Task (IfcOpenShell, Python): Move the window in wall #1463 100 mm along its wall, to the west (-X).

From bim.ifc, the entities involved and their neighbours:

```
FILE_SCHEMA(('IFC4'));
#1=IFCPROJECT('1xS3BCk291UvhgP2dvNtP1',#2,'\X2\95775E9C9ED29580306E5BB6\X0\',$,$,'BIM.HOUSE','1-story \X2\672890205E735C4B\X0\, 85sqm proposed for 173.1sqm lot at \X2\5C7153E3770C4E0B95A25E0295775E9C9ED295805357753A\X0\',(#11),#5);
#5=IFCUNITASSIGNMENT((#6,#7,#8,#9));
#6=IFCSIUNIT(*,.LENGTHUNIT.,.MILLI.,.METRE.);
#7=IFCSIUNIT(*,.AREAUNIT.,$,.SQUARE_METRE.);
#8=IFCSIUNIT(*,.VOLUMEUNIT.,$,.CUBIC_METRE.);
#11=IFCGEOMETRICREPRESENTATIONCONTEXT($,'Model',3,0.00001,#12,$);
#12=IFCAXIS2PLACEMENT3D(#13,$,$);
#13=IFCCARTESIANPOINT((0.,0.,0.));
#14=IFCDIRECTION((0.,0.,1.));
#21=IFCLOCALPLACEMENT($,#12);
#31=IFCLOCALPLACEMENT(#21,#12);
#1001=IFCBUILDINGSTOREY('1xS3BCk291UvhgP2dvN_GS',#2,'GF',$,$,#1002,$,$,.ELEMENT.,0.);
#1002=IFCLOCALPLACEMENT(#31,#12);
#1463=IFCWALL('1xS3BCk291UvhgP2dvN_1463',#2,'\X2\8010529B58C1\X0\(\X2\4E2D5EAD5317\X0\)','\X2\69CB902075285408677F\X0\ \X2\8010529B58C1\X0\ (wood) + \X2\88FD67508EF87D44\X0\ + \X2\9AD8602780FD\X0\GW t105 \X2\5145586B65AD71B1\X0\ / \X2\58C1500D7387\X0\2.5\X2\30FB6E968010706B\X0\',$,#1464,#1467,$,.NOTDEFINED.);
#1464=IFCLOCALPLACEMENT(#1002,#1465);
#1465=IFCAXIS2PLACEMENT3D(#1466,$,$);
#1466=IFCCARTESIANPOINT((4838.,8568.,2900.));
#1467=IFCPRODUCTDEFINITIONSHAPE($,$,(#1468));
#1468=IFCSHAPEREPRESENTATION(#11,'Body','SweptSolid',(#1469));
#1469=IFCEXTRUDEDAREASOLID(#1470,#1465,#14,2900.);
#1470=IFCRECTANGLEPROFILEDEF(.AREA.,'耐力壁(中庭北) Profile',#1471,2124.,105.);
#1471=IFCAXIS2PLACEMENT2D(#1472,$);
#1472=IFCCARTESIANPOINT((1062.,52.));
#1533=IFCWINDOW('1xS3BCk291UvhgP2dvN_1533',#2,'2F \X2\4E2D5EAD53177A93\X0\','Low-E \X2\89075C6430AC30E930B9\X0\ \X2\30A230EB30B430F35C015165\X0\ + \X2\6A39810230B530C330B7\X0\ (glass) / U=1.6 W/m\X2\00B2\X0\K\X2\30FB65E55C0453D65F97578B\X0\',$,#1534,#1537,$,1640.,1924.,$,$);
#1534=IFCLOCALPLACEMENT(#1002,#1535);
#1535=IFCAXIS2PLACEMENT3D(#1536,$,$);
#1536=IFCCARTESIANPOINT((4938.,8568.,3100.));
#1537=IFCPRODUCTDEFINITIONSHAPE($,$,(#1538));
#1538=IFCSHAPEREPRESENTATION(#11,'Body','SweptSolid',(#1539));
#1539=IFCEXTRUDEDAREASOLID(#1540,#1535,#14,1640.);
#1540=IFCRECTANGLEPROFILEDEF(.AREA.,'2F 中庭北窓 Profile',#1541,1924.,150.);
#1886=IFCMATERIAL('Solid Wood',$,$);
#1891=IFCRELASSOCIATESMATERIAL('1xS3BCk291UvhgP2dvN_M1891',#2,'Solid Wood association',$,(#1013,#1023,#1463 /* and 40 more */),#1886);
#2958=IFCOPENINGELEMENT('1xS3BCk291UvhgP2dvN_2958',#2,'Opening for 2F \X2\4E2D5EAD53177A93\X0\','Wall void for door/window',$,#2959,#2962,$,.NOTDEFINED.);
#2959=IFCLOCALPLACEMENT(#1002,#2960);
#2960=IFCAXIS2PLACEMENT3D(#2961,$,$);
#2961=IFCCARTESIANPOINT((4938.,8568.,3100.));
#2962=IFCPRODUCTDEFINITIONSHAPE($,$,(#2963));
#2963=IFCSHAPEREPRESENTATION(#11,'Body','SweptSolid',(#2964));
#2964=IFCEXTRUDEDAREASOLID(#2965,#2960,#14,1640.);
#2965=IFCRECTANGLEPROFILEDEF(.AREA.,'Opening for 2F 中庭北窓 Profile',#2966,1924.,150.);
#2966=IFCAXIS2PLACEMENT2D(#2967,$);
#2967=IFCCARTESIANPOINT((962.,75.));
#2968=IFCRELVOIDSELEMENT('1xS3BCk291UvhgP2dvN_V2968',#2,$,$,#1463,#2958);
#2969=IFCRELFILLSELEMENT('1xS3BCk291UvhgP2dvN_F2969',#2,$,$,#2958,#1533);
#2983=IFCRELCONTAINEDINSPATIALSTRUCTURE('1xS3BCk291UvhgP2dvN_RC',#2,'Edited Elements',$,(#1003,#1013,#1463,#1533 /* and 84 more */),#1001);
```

```python
import ifcopenshell
import ifcopenshell.api.geometry
import ifcopenshell.util.placement
import ifcopenshell.util.unit

model = ifcopenshell.open("bim.ifc")
unit_scale = ifcopenshell.util.unit.calculate_unit_scale(model)

window = model.by_id(1533)
opening = window.FillsVoids[0].RelatingOpeningElement
wall = opening.VoidsElements[0].RelatingBuildingElement

wall_matrix = ifcopenshell.util.placement.get_local_placement(wall.ObjectPlacement)
shift = wall_matrix[:3, 0] * -0.1 / unit_scale
before = ifcopenshell.util.placement.get_local_placement(window.ObjectPlacement)[:3, 3].copy()

# The window is not placed relative to its opening, so move both.
for product in (opening, window):
    matrix = ifcopenshell.util.placement.get_local_placement(product.ObjectPlacement)
    matrix[:3, 3] += shift
    ifcopenshell.api.geometry.edit_object_placement(model, product=product, matrix=matrix, is_si=False)

after = ifcopenshell.util.placement.get_local_placement(window.ObjectPlacement)[:3, 3]
print("window moved by", (after - before).round(3) + 0.0)

model.write("bim_updated.ifc")
```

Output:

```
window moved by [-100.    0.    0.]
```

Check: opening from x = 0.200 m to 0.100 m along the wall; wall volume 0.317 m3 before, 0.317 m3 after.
